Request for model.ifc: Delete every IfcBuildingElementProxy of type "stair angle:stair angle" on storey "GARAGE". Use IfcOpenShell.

First a look at what the model holds.

```python
import ifcopenshell
import ifcopenshell.util.element

model = ifcopenshell.open("model.ifc")
print(model.schema)
storey = next(s for s in model.by_type("IfcBuildingStorey") if s.Name == "GARAGE")
proxies = [e for e in ifcopenshell.util.element.get_decomposition(storey) if e.is_a("IfcBuildingElementProxy")]
seen = {}
for e in proxies:
    element_type = ifcopenshell.util.element.get_type(e)
    name = element_type.Name if element_type not in (None, e) else None
    seen[name] = seen.get(name, 0) + 1
for name, count in sorted(seen.items(), key=str):
    print(count, "x", name)
```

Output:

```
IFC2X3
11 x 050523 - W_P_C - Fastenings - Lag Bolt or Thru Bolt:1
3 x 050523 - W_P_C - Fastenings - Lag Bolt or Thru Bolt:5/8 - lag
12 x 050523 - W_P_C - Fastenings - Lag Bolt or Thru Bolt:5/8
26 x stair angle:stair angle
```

```python
import ifcopenshell
import ifcopenshell.api.root
import ifcopenshell.util.element

model = ifcopenshell.open("model.ifc")

storey = next(s for s in model.by_type("IfcBuildingStorey") if s.Name == "GARAGE")
proxies = [e for e in ifcopenshell.util.element.get_decomposition(storey) if e.is_a("IfcBuildingElementProxy")]
targets = [e for e in proxies if (t := ifcopenshell.util.element.get_type(e)) not in (None, e) and t.Name == "stair angle:stair angle"]

for e in targets:
    ifcopenshell.api.root.remove_product(model, product=e)
print(len(targets), "removed")

model.write("model_updated.ifc")
```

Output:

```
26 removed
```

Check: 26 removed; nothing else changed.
